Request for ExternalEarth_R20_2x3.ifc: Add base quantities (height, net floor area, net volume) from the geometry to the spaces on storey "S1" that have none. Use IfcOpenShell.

First a look at what the model holds.

```python
import ifcopenshell
import ifcopenshell.util.element
import ifcopenshell.util.unit

model = ifcopenshell.open("ExternalEarth_R20_2x3.ifc")
print(model.schema)
for unit_type in ("LENGTHUNIT", "AREAUNIT", "VOLUMEUNIT"):
    print(unit_type, ifcopenshell.util.unit.calculate_unit_scale(model, unit_type))
storey = next(s for s in model.by_type("IfcBuildingStorey") if s.Name == "S1")
spaces = [e for e in ifcopenshell.util.element.get_decomposition(storey) if e.is_a("IfcSpace")]
for e in sorted(spaces, key=lambda e: e.id()):
    print(e.id(), e.is_a(), e.Name, list(ifcopenshell.util.element.get_psets(e, qtos_only=True)), sep=" | ")
```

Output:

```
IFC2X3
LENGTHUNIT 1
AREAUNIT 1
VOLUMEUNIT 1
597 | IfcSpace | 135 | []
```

```python
import ifcopenshell
import ifcopenshell.api.pset
import ifcopenshell.geom
import ifcopenshell.util.element
import ifcopenshell.util.shape
import ifcopenshell.util.unit

model = ifcopenshell.open("ExternalEarth_R20_2x3.ifc")
unit_scale = ifcopenshell.util.unit.calculate_unit_scale(model)
area_scale = ifcopenshell.util.unit.calculate_unit_scale(model, "AREAUNIT")
volume_scale = ifcopenshell.util.unit.calculate_unit_scale(model, "VOLUMEUNIT")
settings = ifcopenshell.geom.settings()

storey = next(s for s in model.by_type("IfcBuildingStorey") if s.Name == "S1")
spaces = [e for e in ifcopenshell.util.element.get_decomposition(storey) if e.is_a("IfcSpace")]

for e in sorted(spaces, key=lambda e: e.id()):
    if ifcopenshell.util.element.get_psets(e, qtos_only=True, should_inherit=False):
        continue
    # Geometry comes back in metres, in the element's own axes.
    shape = ifcopenshell.geom.create_shape(settings, e)
    values = {
        "Height": ifcopenshell.util.shape.get_z(shape.geometry) / unit_scale,
        "NetFloorArea": ifcopenshell.util.shape.get_footprint_area(shape.geometry) / area_scale,
        "NetVolume": ifcopenshell.util.shape.get_volume(shape.geometry) / volume_scale,
    }
    qto = ifcopenshell.api.pset.add_qto(model, product=e, name="BaseQuantities")
    ifcopenshell.api.pset.edit_qto(model, qto=qto, properties=values)
    print(e.id(), {k: round(v, 3) for k, v in values.items()})

model.write("ExternalEarth_R20_2x3_rev.ifc")
```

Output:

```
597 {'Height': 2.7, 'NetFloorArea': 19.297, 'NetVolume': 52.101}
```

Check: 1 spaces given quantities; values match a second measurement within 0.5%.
